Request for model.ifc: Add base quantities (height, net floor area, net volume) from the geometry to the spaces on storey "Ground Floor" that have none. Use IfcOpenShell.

First a look at what the model holds.

```python
import ifcopenshell
import ifcopenshell.util.element
import ifcopenshell.util.unit

model = ifcopenshell.open("model.ifc")
print(model.schema)
for unit_type in ("LENGTHUNIT", "AREAUNIT", "VOLUMEUNIT"):
    print(unit_type, ifcopenshell.util.unit.calculate_unit_scale(model, unit_type))
storey = next(s for s in model.by_type("IfcBuildingStorey") if s.Name == "Ground Floor")
spaces = [e for e in ifcopenshell.util.element.get_decomposition(storey) if e.is_a("IfcSpace")]
for e in sorted(spaces, key=lambda e: e.id()):
    print(e.id(), e.is_a(), e.Name, list(ifcopenshell.util.element.get_psets(e, qtos_only=True)), sep=" | ")
```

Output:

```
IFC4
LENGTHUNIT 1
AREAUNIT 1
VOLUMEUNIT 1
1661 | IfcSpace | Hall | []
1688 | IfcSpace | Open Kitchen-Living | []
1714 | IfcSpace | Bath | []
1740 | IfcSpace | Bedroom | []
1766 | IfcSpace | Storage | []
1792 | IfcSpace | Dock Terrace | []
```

```python
import ifcopenshell
import ifcopenshell.api.pset
import ifcopenshell.geom
import ifcopenshell.util.element
import ifcopenshell.util.shape
import ifcopenshell.util.unit

model = ifcopenshell.open("model.ifc")
unit_scale = ifcopenshell.util.unit.calculate_unit_scale(model)
area_scale = ifcopenshell.util.unit.calculate_unit_scale(model, "AREAUNIT")
volume_scale = ifcopenshell.util.unit.calculate_unit_scale(model, "VOLUMEUNIT")
settings = ifcopenshell.geom.settings()

storey = next(s for s in model.by_type("IfcBuildingStorey") if s.Name == "Ground Floor")
spaces = [e for e in ifcopenshell.util.element.get_decomposition(storey) if e.is_a("IfcSpace")]

for e in sorted(spaces, key=lambda e: e.id()):
    if ifcopenshell.util.element.get_psets(e, qtos_only=True, should_inherit=False):
        continue
    # Geometry comes back in metres, in the element's own axes.
    shape = ifcopenshell.geom.create_shape(settings, e)
    values = {
        "Height": ifcopenshell.util.shape.get_z(shape.geometry) / unit_scale,
        "NetFloorArea": ifcopenshell.util.shape.get_footprint_area(shape.geometry) / area_scale,
        "NetVolume": ifcopenshell.util.shape.get_volume(shape.geometry) / volume_scale,
    }
    qto = ifcopenshell.api.pset.add_qto(model, product=e, name="Qto_SpaceBaseQuantities")
    ifcopenshell.api.pset.edit_qto(model, qto=qto, properties=values)
    print(e.id(), {k: round(v, 3) for k, v in values.items()})

model.write("model-out.ifc")
```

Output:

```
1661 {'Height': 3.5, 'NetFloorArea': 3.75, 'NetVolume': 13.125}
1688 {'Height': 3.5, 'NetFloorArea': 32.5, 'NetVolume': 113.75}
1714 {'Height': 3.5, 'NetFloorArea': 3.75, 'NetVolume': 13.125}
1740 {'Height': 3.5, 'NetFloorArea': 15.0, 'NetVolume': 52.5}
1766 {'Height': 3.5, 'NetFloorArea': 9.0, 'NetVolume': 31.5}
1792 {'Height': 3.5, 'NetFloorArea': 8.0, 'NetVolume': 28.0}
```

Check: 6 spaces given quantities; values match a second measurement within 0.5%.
